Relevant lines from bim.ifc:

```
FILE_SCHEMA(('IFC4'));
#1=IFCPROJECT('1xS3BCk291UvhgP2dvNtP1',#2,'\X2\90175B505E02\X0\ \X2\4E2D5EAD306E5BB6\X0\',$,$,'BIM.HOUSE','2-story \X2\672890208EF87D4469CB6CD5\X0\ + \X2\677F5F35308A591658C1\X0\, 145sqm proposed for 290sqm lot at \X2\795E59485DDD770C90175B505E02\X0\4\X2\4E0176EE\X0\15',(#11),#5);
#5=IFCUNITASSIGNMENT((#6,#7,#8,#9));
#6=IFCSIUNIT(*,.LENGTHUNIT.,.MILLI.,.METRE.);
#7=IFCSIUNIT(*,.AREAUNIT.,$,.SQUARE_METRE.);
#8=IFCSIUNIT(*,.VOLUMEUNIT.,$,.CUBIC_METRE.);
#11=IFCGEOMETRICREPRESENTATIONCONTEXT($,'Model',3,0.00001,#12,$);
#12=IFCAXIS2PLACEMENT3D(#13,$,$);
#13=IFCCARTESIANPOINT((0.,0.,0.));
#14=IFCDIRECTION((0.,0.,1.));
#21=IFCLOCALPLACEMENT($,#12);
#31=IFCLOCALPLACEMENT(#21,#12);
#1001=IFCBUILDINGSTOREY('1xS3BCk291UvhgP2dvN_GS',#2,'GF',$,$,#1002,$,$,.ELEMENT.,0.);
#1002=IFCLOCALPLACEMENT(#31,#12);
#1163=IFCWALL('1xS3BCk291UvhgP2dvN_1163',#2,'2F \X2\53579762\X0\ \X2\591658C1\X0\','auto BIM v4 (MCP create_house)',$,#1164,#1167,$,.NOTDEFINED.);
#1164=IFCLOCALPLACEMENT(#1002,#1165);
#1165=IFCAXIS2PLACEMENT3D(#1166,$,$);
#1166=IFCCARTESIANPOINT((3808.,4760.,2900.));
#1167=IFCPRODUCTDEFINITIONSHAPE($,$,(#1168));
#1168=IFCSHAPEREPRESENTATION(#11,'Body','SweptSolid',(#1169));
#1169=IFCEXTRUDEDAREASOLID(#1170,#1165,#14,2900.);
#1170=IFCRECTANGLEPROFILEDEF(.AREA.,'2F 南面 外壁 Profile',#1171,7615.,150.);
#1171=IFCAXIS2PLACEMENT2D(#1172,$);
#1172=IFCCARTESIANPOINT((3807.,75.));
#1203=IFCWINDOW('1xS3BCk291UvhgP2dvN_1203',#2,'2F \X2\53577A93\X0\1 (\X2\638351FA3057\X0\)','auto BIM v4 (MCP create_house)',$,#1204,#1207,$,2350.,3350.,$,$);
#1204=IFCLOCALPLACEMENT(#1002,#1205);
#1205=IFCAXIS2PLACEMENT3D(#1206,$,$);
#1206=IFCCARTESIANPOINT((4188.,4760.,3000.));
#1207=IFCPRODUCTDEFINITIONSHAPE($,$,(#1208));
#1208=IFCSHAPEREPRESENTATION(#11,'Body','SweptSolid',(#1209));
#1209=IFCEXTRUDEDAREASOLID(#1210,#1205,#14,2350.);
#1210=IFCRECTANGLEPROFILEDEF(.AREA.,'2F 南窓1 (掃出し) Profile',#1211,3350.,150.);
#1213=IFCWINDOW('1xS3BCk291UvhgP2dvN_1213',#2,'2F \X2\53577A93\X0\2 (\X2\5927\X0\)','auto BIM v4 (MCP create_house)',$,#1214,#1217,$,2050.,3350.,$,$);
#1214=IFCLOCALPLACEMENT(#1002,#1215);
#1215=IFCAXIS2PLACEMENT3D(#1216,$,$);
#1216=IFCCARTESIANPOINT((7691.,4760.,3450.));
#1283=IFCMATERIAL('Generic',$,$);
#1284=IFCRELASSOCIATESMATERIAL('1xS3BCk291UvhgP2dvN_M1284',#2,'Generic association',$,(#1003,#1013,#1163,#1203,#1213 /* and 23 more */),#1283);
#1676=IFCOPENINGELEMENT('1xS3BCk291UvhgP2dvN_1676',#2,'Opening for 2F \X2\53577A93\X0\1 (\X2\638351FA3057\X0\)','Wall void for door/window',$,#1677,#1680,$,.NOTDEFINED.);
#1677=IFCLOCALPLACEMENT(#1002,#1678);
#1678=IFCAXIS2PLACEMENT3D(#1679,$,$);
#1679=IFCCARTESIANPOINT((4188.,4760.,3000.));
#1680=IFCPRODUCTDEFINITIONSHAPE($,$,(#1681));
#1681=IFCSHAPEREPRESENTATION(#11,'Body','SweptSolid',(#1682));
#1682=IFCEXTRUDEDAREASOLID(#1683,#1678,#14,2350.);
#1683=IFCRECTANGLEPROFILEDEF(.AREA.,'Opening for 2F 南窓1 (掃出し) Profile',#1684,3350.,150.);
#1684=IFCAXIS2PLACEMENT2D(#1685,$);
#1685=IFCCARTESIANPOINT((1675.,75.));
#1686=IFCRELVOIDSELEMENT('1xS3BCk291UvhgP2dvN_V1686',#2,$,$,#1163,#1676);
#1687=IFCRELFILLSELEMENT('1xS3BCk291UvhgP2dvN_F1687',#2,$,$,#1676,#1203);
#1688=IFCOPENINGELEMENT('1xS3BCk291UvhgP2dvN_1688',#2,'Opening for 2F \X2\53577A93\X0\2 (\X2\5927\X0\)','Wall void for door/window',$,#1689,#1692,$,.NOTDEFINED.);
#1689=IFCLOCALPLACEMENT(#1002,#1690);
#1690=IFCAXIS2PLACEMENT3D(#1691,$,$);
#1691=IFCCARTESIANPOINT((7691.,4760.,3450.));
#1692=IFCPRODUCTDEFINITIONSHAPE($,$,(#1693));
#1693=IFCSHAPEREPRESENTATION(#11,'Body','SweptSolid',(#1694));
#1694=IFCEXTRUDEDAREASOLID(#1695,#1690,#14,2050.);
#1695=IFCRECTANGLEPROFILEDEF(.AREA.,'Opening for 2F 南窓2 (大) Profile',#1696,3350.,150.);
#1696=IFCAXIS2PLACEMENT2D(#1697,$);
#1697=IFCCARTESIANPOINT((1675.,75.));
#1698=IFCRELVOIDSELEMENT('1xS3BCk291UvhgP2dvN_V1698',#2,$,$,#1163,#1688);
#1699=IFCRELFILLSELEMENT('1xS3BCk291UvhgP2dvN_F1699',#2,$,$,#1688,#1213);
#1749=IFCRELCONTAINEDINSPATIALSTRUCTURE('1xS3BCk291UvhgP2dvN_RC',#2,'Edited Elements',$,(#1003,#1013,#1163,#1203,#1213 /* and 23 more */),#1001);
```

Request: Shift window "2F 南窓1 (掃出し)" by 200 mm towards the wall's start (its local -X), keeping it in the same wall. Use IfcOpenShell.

```python
import ifcopenshell
import ifcopenshell.api.geometry
import ifcopenshell.util.placement

model = ifcopenshell.open("bim.ifc")

window = model.by_id(1203)
opening = window.FillsVoids[0].RelatingOpeningElement
wall = opening.VoidsElements[0].RelatingBuildingElement

wall_matrix = ifcopenshell.util.placement.get_local_placement(wall.ObjectPlacement)
shift = wall_matrix[:3, 0] * -200.0
before = ifcopenshell.util.placement.get_local_placement(window.ObjectPlacement)[:3, 3].copy()

# The window is not placed relative to its opening, so move both.
for product in (opening, window):
    matrix = ifcopenshell.util.placement.get_local_placement(product.ObjectPlacement)
    matrix[:3, 3] += shift
    ifcopenshell.api.geometry.edit_object_placement(model, product=product, matrix=matrix, is_si=False)

after = ifcopenshell.util.placement.get_local_placement(window.ObjectPlacement)[:3, 3]
print("window moved by", (after - before).round(3) + 0.0)

model.write("bim_edited.ifc")
```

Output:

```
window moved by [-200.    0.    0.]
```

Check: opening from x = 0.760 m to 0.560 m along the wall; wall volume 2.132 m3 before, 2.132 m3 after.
